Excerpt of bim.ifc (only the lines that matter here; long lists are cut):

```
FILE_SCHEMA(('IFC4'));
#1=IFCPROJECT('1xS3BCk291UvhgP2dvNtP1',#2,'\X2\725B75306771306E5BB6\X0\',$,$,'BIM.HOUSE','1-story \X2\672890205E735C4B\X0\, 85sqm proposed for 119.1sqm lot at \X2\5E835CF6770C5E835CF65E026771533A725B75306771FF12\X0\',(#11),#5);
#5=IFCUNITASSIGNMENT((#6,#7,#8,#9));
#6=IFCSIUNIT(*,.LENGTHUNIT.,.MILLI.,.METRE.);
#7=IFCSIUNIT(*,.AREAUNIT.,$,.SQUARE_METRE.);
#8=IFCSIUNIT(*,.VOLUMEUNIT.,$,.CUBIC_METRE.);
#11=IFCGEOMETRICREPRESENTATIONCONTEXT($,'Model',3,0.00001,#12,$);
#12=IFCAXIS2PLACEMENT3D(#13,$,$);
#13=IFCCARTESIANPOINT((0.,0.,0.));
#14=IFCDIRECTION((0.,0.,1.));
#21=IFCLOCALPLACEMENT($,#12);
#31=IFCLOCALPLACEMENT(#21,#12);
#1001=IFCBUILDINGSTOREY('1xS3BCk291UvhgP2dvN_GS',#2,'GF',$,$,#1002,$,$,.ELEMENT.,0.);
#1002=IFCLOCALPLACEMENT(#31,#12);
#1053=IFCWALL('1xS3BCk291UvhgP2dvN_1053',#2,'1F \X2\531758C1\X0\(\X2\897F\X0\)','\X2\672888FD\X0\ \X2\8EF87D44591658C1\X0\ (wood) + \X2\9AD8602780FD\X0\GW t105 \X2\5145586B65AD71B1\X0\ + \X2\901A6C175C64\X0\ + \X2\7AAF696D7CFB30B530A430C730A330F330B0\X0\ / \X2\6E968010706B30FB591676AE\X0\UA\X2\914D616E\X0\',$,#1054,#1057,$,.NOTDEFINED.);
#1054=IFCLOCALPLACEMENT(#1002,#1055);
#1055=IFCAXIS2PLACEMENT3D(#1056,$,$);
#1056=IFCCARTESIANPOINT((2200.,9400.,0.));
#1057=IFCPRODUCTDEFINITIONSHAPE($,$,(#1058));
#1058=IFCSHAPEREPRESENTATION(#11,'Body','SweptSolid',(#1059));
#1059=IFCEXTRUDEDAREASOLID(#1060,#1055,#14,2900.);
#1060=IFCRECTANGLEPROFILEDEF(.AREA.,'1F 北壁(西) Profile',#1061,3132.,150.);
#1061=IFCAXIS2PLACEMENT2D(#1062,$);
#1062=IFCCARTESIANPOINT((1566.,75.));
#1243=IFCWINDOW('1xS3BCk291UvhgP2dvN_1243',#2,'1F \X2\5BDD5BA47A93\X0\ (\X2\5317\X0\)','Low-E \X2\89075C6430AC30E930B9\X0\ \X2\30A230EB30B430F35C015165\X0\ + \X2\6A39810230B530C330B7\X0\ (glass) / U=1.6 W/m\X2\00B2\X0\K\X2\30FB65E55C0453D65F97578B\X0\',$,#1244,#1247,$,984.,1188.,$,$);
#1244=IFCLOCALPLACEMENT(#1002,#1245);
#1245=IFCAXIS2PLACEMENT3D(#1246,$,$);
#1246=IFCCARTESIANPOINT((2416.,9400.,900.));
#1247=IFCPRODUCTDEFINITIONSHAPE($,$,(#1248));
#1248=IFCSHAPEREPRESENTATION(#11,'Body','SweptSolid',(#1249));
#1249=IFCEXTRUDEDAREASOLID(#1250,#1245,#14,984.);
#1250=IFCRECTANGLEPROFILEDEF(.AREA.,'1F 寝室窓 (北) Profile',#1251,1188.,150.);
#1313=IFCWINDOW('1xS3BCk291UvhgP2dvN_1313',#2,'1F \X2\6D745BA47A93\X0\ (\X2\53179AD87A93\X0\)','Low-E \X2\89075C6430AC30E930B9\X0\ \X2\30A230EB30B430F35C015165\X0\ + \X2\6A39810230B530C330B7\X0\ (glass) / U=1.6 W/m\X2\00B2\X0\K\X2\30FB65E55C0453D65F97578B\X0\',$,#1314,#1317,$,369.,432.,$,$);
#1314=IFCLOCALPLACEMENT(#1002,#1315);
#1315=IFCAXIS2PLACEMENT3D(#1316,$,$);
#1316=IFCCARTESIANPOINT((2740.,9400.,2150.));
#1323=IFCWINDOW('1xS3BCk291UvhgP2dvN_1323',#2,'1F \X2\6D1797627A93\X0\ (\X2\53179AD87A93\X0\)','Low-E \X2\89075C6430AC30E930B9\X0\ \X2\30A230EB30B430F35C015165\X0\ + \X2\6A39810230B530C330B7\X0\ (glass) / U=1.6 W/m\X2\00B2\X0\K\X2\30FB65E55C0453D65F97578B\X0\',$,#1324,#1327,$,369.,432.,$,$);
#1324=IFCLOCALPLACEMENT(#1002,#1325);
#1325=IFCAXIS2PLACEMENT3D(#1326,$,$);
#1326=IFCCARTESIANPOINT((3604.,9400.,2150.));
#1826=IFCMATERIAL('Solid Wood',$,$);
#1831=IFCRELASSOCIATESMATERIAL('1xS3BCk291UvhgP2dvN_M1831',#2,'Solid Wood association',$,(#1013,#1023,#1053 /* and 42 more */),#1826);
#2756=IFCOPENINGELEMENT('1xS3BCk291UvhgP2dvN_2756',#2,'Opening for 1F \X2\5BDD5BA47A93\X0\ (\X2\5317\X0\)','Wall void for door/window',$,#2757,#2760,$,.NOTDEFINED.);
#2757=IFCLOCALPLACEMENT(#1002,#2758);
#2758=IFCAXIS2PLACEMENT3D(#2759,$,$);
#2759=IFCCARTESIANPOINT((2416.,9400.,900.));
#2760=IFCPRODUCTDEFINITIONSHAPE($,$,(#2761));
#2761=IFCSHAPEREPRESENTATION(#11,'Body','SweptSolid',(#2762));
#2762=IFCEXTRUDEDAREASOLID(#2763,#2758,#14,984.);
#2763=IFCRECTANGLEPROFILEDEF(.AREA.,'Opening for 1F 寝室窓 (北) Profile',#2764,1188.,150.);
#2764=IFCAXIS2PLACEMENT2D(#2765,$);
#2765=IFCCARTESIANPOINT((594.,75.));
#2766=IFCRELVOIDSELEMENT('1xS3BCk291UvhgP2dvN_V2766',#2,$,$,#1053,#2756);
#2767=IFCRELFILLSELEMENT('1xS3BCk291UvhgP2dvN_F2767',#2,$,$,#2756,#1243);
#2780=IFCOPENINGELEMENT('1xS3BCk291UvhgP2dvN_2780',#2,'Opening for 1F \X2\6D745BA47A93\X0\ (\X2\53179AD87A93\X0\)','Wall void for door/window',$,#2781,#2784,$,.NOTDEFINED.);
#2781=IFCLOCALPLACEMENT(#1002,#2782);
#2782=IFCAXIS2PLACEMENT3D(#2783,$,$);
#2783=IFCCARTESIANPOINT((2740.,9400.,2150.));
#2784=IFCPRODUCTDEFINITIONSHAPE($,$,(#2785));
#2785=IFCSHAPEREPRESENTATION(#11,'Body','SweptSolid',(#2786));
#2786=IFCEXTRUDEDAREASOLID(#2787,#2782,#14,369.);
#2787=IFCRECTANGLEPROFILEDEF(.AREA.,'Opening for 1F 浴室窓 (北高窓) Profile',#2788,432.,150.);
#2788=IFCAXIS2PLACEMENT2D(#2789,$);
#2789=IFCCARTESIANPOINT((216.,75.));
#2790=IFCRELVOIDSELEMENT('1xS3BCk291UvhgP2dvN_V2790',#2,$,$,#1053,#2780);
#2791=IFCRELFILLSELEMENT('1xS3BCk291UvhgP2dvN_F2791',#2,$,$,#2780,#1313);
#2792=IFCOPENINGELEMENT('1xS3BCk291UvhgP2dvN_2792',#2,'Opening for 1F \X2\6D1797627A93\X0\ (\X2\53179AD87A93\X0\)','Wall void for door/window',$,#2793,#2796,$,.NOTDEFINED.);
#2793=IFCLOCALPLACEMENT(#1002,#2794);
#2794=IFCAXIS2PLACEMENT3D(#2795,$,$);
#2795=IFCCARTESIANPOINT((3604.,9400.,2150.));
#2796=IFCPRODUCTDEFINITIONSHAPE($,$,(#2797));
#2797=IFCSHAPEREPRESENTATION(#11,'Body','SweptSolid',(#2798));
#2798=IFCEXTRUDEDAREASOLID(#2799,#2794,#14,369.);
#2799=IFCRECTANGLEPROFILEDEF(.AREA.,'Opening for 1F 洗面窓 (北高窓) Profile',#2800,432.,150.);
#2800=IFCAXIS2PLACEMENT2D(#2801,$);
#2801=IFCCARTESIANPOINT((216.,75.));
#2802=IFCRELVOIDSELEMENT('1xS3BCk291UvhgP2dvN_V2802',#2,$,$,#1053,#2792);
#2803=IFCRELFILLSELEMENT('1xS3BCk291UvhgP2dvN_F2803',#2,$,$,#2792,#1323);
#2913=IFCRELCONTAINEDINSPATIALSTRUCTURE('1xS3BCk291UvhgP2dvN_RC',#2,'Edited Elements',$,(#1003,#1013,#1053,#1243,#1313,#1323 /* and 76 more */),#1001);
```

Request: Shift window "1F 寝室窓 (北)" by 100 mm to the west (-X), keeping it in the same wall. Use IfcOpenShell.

```python
import ifcopenshell
import ifcopenshell.api.geometry
import ifcopenshell.util.placement
import ifcopenshell.util.unit

model = ifcopenshell.open("bim.ifc")
unit_scale = ifcopenshell.util.unit.calculate_unit_scale(model)

window = model.by_guid("1xS3BCk291UvhgP2dvN_1243")
opening = window.FillsVoids[0].RelatingOpeningElement
wall = opening.VoidsElements[0].RelatingBuildingElement

wall_matrix = ifcopenshell.util.placement.get_local_placement(wall.ObjectPlacement)
shift = wall_matrix[:3, 0] * -0.1 / unit_scale
before = ifcopenshell.util.placement.get_local_placement(window.ObjectPlacement)[:3, 3].copy()

# The window is not placed relative to its opening, so move both.
for product in (opening, window):
    matrix = ifcopenshell.util.placement.get_local_placement(product.ObjectPlacement)
    matrix[:3, 3] += shift
    ifcopenshell.api.geometry.edit_object_placement(model, product=product, matrix=matrix, is_si=False)

after = ifcopenshell.util.placement.get_local_placement(window.ObjectPlacement)[:3, 3]
print("window moved by", (after - before).round(3) + 0.0)

model.write("bim_updated.ifc")
```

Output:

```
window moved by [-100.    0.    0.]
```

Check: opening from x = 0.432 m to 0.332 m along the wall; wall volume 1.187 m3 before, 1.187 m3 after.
